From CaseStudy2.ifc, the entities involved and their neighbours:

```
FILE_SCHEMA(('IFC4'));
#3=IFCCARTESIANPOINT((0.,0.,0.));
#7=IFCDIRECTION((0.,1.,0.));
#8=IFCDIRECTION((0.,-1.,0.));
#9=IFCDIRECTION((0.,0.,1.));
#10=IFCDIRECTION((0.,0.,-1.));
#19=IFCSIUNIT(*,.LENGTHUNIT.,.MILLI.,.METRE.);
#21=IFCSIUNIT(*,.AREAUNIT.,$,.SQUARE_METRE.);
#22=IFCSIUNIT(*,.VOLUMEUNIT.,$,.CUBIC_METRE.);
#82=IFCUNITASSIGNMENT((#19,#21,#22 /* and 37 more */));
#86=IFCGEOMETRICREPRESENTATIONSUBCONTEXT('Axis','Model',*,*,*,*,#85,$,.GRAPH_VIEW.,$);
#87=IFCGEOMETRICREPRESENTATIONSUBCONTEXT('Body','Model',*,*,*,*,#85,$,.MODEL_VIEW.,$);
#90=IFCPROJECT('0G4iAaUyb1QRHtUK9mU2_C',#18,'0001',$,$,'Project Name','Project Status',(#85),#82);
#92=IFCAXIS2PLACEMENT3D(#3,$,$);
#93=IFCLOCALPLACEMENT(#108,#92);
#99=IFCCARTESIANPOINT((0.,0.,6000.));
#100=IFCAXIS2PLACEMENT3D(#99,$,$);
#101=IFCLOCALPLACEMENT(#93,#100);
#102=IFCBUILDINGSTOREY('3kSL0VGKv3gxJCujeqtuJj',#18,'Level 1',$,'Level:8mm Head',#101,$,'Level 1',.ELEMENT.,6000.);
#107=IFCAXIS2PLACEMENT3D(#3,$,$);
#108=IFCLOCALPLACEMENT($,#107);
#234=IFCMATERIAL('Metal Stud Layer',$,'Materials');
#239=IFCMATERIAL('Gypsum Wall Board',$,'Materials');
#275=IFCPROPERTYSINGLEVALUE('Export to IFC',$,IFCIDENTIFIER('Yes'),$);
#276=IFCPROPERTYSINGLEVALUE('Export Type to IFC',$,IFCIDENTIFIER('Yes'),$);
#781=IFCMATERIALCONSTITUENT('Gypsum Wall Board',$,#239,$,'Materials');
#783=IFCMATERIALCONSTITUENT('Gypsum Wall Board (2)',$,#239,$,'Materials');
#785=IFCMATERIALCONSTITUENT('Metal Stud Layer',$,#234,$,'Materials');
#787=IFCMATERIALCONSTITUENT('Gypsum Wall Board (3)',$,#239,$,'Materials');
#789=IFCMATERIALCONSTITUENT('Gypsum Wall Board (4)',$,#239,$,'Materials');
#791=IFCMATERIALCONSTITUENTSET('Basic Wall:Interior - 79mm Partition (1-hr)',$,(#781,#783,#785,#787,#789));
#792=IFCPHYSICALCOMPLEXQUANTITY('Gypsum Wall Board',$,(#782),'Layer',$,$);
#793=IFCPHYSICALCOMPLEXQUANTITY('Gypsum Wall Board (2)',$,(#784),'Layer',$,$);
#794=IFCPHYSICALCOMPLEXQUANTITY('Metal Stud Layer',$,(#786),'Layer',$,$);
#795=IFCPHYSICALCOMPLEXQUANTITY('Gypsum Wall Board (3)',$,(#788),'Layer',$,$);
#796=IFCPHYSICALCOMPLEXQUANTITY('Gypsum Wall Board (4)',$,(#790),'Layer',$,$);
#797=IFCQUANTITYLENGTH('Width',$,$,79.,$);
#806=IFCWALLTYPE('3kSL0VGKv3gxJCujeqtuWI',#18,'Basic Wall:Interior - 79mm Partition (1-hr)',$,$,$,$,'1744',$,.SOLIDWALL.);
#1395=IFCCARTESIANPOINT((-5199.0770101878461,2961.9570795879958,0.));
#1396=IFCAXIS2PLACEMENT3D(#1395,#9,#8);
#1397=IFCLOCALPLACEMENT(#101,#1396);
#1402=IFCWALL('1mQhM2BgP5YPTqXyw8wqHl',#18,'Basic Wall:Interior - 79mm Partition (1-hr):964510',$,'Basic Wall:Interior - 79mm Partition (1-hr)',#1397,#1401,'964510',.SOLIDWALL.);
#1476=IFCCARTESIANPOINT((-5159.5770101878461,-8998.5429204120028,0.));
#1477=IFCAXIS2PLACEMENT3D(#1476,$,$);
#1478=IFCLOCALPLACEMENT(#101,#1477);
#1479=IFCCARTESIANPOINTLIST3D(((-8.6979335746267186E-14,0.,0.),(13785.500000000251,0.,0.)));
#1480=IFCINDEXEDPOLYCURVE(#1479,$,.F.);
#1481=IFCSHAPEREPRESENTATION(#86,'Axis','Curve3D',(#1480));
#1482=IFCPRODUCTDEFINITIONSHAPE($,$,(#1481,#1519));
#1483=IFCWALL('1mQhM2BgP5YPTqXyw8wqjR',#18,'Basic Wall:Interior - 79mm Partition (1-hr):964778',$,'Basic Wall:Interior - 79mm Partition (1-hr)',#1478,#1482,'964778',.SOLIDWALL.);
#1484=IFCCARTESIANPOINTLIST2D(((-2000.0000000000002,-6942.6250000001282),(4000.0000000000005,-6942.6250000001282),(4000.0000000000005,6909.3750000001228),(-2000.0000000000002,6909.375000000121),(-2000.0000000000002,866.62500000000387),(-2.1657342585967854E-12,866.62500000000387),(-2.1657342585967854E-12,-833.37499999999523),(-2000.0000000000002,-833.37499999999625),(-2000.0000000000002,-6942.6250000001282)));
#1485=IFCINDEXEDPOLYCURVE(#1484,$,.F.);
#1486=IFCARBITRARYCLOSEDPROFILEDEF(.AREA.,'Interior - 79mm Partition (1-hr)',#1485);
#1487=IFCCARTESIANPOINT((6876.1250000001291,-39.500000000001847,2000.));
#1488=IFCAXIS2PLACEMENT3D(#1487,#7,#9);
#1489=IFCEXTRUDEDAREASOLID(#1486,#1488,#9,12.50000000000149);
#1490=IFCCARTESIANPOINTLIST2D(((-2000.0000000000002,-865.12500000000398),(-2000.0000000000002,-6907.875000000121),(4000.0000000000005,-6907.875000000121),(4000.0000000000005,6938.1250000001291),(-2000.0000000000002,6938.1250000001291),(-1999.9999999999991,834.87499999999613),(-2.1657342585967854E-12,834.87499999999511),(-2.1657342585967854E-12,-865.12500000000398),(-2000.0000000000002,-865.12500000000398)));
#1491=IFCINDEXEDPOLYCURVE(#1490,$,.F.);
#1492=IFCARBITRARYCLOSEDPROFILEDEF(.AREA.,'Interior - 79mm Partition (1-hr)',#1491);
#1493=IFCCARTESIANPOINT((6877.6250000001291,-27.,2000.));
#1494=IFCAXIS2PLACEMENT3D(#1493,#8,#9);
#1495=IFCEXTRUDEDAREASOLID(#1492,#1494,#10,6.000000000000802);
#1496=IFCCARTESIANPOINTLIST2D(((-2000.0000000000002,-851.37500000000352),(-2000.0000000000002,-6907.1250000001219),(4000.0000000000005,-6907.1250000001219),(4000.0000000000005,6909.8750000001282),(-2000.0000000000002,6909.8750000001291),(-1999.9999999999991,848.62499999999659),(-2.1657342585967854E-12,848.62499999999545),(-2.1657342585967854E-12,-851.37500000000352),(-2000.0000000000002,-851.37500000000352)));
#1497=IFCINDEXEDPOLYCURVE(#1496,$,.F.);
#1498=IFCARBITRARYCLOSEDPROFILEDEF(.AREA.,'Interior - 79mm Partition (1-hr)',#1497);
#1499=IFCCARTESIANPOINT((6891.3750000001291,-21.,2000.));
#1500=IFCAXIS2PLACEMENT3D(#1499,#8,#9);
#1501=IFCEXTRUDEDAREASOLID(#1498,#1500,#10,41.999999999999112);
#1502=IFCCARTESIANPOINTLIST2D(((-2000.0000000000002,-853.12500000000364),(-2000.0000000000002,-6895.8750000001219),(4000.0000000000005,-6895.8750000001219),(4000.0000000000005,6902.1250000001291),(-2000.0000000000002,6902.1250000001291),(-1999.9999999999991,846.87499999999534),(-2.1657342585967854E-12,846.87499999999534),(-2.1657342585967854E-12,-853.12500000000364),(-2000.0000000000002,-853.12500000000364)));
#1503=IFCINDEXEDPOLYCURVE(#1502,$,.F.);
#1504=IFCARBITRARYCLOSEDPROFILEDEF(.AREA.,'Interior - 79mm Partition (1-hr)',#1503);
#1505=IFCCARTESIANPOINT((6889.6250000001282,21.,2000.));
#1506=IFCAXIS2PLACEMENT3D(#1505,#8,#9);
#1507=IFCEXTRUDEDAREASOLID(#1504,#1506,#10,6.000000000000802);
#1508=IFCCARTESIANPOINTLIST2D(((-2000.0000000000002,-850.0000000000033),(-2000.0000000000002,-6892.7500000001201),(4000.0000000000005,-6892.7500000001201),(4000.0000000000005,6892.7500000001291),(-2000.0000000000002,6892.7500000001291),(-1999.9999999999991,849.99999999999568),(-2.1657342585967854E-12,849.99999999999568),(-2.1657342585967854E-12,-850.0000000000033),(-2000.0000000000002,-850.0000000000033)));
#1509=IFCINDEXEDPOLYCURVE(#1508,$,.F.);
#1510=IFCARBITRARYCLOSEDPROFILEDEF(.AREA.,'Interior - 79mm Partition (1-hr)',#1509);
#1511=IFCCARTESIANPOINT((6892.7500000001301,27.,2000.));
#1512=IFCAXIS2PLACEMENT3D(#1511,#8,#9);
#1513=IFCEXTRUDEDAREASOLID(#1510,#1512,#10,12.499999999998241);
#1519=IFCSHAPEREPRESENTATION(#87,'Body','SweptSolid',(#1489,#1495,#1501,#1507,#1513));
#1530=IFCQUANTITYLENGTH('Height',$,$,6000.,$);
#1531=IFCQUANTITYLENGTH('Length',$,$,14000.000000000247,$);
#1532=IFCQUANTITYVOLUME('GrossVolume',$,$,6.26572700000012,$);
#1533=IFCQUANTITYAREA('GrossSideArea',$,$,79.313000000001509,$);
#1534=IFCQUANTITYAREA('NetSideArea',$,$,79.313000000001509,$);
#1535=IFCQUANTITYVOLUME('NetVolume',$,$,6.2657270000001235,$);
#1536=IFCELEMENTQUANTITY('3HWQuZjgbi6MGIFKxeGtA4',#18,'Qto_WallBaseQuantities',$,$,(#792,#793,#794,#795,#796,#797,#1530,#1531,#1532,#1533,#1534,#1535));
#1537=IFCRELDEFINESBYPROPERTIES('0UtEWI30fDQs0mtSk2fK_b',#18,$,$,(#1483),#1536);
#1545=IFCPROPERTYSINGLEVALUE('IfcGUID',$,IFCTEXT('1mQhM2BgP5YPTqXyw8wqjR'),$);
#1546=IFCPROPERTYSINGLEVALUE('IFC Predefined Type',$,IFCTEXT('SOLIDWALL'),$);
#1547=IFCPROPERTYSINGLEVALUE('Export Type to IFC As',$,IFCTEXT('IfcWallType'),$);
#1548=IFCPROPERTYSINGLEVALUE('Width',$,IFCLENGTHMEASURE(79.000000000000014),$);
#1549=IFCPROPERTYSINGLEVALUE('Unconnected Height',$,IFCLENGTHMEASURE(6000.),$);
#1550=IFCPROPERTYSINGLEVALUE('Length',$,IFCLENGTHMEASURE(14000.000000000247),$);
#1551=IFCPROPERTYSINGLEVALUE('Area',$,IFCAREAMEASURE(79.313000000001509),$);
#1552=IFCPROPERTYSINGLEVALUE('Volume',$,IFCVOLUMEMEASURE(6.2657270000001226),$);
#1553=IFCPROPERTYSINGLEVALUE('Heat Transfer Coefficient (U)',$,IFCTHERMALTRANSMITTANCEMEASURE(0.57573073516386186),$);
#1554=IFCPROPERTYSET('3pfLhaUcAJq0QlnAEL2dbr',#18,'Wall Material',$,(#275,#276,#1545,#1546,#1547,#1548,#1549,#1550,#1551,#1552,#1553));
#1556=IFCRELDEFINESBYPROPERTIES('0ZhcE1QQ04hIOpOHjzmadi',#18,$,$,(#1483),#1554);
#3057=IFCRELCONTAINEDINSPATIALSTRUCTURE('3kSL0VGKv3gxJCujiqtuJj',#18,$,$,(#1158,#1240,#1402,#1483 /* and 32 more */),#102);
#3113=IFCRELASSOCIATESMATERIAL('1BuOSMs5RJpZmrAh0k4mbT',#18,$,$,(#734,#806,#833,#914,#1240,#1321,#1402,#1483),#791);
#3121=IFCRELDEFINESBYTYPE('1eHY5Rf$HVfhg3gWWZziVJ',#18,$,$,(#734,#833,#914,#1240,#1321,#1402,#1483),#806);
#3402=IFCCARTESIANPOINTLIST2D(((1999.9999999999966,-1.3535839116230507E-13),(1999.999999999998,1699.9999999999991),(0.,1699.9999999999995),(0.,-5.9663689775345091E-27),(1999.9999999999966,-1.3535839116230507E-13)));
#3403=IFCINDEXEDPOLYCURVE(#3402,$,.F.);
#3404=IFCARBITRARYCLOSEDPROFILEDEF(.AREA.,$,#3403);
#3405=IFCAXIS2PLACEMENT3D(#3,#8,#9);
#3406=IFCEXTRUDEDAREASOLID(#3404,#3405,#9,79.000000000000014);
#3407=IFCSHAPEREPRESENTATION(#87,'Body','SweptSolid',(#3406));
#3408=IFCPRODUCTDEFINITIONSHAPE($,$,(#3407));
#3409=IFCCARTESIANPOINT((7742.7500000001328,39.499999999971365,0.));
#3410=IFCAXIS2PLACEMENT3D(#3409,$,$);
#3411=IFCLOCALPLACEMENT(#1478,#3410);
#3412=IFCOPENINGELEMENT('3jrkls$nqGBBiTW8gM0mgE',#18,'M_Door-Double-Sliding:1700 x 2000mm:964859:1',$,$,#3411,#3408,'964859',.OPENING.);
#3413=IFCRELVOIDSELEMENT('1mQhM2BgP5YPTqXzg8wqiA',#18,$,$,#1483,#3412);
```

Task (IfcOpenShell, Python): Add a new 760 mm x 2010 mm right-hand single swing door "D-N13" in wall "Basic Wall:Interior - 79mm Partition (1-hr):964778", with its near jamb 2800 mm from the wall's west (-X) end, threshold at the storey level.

```python
import numpy as np
import ifcopenshell
import ifcopenshell.api.feature
import ifcopenshell.api.geometry
import ifcopenshell.api.pset
import ifcopenshell.api.root
import ifcopenshell.api.spatial
import ifcopenshell.geom
import ifcopenshell.util.element
import ifcopenshell.util.placement
import ifcopenshell.util.representation
import ifcopenshell.util.shape
import ifcopenshell.util.unit

model = ifcopenshell.open("CaseStudy2.ifc")
unit_scale = ifcopenshell.util.unit.calculate_unit_scale(model)
area_scale = ifcopenshell.util.unit.calculate_unit_scale(model, "AREAUNIT")
volume_scale = ifcopenshell.util.unit.calculate_unit_scale(model, "VOLUMEUNIT")
settings = ifcopenshell.geom.settings()


def volume(element):
    """Net volume in cubic metres, openings subtracted."""
    shape = ifcopenshell.geom.create_shape(settings, element)
    return ifcopenshell.util.shape.get_volume(shape.geometry)


wall = model.by_guid("1mQhM2BgP5YPTqXyw8wqjR")
storey = ifcopenshell.util.element.get_container(wall, ifc_class="IfcBuildingStorey")
context = ifcopenshell.util.representation.get_context(model, "Model", "Body", "MODEL_VIEW")
before = volume(wall)

width, height, from_end, sill = 0.76, 2.01, 2.8, 0.0  # metres

# The wall runs along its own X axis, and the end named is its -X end.
wall_shape = ifcopenshell.geom.create_shape(settings, wall)
x, y, z = ifcopenshell.util.shape.get_vertices(wall_shape.geometry).T
start = x.min() + from_end
face, thickness = float(y.min()), float(y.max() - y.min())
wall_matrix = ifcopenshell.util.placement.get_local_placement(wall.ObjectPlacement)
level = ifcopenshell.util.placement.get_local_placement(storey.ObjectPlacement)[2, 3]


def in_wall(x, y):
    """Placement at x, y metres in the wall's axes, at sill height."""
    matrix = wall_matrix.copy()
    matrix[:, 3] = wall_matrix @ np.array([x / unit_scale, y / unit_scale, 0.0, 1.0])
    matrix[2, 3] = level + sill / unit_scale
    return matrix


# Opening: a box that overshoots both wall faces by 50 mm.
opening = ifcopenshell.api.root.create_entity(model, ifc_class="IfcOpeningElement", predefined_type="OPENING")
box = ifcopenshell.api.geometry.add_wall_representation(
    model, context=context, length=width, height=height, thickness=thickness + 0.1
)
ifcopenshell.api.geometry.assign_representation(model, product=opening, representation=box)
ifcopenshell.api.geometry.edit_object_placement(model, product=opening, matrix=in_wall(start, face - 0.05), is_si=False)
ifcopenshell.api.feature.add_feature(model, feature=opening, element=wall)

door = ifcopenshell.api.root.create_entity(model, ifc_class="IfcDoor", name="D-N13", predefined_type="DOOR")
door.OverallWidth, door.OverallHeight = width / unit_scale, height / unit_scale
door.OperationType = "SINGLE_SWING_RIGHT"
body = ifcopenshell.api.geometry.add_door_representation(
    model,
    context=context,
    overall_width=door.OverallWidth,
    overall_height=door.OverallHeight,
    operation_type="SINGLE_SWING_RIGHT",
    lining_properties={"LiningDepth": thickness / unit_scale, "ThresholdDepth": thickness / unit_scale},
)
ifcopenshell.api.geometry.assign_representation(model, product=door, representation=body)
ifcopenshell.api.spatial.assign_container(model, products=[door], relating_structure=storey)
ifcopenshell.api.feature.add_filling(model, opening=opening, element=door)

# The lining spans the wall, so the door starts at the wall face.
ifcopenshell.api.geometry.edit_object_placement(model, product=door, matrix=in_wall(start, face), is_si=False)

after = volume(wall)

# Update the wall's stored quantities.
qto = model.by_id(ifcopenshell.util.element.get_pset(wall, "Qto_WallBaseQuantities", should_inherit=False)["id"])
ifcopenshell.api.pset.edit_qto(model, qto=qto, properties={
    "NetSideArea": after / thickness / area_scale,
    "NetVolume": after / volume_scale,
})
pset = model.by_id(ifcopenshell.util.element.get_pset(wall, "Wall Material", should_inherit=False)["id"])
ifcopenshell.api.pset.edit_pset(model, pset=pset, properties={
    "Area": model.create_entity("IfcAreaMeasure", after / thickness / area_scale),
    "Volume": model.create_entity("IfcVolumeMeasure", after / volume_scale),
})

print(f"wall volume {before:.3f} -> {after:.3f} m3")

model.write("CaseStudy2_rev.ifc")
```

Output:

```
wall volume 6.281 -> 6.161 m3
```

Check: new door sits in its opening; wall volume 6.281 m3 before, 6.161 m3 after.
